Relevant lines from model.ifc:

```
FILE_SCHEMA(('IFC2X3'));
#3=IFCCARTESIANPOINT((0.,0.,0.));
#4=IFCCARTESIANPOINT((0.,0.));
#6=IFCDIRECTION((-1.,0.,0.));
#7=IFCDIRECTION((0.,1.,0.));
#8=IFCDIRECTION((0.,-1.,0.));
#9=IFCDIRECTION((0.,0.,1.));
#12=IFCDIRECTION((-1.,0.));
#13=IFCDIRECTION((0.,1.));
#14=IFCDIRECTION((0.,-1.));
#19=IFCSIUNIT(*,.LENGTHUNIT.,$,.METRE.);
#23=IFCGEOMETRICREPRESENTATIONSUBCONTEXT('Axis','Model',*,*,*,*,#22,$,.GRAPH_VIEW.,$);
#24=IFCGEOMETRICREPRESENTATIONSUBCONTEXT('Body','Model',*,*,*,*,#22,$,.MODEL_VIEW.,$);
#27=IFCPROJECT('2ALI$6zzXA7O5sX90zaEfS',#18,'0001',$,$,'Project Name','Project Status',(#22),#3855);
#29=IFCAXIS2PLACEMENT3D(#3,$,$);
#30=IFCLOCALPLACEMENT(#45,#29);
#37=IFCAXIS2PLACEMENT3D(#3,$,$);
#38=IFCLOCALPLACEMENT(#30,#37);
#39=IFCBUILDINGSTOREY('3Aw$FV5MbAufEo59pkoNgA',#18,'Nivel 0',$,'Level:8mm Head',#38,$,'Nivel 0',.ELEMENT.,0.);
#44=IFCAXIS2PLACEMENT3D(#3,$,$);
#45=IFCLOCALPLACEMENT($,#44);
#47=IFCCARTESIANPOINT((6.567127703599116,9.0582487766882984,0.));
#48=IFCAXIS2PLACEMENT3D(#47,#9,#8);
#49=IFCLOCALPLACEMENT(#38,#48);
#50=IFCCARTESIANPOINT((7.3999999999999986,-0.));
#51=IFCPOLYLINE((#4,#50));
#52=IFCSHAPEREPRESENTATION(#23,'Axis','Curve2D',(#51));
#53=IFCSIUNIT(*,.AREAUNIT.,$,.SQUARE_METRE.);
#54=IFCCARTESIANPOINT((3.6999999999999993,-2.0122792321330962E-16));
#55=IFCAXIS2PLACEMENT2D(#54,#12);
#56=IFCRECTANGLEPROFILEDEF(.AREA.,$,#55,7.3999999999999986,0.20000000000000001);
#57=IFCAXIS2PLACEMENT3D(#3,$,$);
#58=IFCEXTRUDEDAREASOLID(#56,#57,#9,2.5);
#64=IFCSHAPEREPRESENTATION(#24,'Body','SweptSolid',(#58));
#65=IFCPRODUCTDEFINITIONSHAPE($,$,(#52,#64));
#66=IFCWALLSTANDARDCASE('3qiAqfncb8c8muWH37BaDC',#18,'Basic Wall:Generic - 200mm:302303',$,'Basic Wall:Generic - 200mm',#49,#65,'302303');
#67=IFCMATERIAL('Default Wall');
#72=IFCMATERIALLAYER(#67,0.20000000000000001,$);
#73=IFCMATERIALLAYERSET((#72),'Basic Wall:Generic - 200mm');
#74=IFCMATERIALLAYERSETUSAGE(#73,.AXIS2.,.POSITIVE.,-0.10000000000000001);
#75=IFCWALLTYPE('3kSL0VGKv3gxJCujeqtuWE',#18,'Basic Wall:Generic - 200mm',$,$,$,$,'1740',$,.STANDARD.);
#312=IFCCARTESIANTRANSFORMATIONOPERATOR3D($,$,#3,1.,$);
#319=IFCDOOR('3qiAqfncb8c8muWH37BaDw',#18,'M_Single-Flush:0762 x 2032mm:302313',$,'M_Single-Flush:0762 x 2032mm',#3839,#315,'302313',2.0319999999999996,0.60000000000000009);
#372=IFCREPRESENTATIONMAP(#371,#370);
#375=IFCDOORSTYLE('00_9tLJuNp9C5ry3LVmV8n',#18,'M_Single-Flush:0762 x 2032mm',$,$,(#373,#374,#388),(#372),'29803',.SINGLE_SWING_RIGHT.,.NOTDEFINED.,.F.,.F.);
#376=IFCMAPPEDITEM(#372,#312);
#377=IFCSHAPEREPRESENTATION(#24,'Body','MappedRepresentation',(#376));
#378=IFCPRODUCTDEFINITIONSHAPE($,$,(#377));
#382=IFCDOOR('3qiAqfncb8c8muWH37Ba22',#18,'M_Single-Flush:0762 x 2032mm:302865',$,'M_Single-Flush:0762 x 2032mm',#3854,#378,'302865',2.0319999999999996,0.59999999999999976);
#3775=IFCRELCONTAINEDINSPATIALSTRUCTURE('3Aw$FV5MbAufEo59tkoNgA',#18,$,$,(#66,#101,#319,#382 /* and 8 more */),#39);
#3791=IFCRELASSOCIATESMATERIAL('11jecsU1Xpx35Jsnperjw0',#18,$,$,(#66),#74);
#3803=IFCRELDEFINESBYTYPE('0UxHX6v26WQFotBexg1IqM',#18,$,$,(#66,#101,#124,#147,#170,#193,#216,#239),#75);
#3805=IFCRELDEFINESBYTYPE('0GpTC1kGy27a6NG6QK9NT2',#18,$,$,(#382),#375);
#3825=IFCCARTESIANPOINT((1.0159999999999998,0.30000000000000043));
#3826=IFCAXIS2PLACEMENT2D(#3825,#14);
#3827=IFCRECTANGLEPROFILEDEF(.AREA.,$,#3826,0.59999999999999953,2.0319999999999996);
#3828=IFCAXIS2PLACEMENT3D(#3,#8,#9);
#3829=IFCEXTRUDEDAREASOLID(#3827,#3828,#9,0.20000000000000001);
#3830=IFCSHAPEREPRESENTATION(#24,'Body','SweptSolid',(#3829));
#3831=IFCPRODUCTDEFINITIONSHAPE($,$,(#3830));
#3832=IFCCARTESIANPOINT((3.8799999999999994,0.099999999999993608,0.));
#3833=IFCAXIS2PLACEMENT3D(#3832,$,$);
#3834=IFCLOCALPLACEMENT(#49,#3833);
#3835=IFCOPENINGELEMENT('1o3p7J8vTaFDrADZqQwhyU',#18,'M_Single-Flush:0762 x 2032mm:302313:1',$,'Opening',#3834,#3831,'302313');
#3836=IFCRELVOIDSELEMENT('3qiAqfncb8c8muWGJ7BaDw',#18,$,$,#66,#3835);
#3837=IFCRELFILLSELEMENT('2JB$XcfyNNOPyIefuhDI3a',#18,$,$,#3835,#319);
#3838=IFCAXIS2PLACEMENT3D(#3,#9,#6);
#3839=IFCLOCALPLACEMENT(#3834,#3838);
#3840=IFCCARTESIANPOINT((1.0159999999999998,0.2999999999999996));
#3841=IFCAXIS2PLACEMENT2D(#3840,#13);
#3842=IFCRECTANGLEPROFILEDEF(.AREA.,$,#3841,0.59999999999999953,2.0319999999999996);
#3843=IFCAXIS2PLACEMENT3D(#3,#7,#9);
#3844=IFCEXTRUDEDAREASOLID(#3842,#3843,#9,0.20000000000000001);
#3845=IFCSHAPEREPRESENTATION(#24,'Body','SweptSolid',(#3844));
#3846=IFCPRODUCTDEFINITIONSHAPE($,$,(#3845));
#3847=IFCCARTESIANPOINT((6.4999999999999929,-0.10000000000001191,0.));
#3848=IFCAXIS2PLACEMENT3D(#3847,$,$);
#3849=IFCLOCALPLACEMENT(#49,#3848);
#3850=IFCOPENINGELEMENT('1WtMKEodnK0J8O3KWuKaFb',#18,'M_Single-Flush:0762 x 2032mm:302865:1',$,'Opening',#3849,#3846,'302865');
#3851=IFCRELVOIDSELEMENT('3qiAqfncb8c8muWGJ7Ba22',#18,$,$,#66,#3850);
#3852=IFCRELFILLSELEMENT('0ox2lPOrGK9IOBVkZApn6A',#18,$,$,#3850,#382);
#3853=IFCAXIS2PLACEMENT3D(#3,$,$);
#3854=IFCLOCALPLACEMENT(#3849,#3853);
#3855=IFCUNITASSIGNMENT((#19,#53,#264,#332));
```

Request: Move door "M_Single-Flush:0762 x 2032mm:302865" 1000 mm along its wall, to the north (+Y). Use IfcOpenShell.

```python
import ifcopenshell
import ifcopenshell.api.geometry
import ifcopenshell.util.placement
import ifcopenshell.util.unit

model = ifcopenshell.open("model.ifc")
unit_scale = ifcopenshell.util.unit.calculate_unit_scale(model)

door = model.by_guid("3qiAqfncb8c8muWH37Ba22")
opening = door.FillsVoids[0].RelatingOpeningElement
wall = opening.VoidsElements[0].RelatingBuildingElement

wall_matrix = ifcopenshell.util.placement.get_local_placement(wall.ObjectPlacement)
shift = wall_matrix[:3, 0] * -1 / unit_scale
before = ifcopenshell.util.placement.get_local_placement(door.ObjectPlacement)[:3, 3].copy()

# The door is placed relative to its opening, so it follows when the opening moves.
matrix = ifcopenshell.util.placement.get_local_placement(opening.ObjectPlacement)
matrix[:3, 3] += shift
ifcopenshell.api.geometry.edit_object_placement(
    model, product=opening, matrix=matrix, is_si=False, should_transform_children=True
)

after = ifcopenshell.util.placement.get_local_placement(door.ObjectPlacement)[:3, 3]
print("door moved by", (after - before).round(3) + 0.0)

model.write("model-out.ifc")
```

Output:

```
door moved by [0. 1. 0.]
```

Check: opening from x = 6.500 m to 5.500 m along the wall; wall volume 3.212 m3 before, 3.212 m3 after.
